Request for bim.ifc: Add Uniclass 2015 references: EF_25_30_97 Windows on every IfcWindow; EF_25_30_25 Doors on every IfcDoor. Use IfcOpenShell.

First a look at what the model holds.

```python
import ifcopenshell

model = ifcopenshell.open("bim.ifc")
print(model.schema)
print("classifications:", [c.Name for c in model.by_type("IfcClassification")])
for ifc_class in ("IfcDoor", "IfcRoof", "IfcStair", "IfcWall", "IfcWindow"):
    print(ifc_class, len(model.by_type(ifc_class)))
```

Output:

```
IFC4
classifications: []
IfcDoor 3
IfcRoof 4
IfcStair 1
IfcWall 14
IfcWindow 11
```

```python
import ifcopenshell
import ifcopenshell.api.classification

model = ifcopenshell.open("bim.ifc")

system = ifcopenshell.api.classification.add_classification(model, classification="Uniclass 2015")

codes = {
    "IfcWindow": ("EF_25_30_97", "Windows"),
    "IfcDoor": ("EF_25_30_25", "Doors"),
}
for ifc_class, (code, name) in codes.items():
    products = model.by_type(ifc_class)
    ifcopenshell.api.classification.add_reference(
        model, products=products, classification=system, identification=code, name=name
    )
    print(code, len(products))

model.write("bim_edited.ifc")
```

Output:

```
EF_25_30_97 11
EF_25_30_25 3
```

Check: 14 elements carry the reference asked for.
